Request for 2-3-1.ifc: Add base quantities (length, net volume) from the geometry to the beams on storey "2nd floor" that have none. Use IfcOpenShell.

First a look at what the model holds.

```python
import ifcopenshell
import ifcopenshell.util.element
import ifcopenshell.util.unit

model = ifcopenshell.open("2-3-1.ifc")
print(model.schema)
for unit_type in ("LENGTHUNIT", "AREAUNIT", "VOLUMEUNIT"):
    print(unit_type, ifcopenshell.util.unit.calculate_unit_scale(model, unit_type))
storey = next(s for s in model.by_type("IfcBuildingStorey") if s.Name == "2nd floor")
beams = [e for e in ifcopenshell.util.element.get_decomposition(storey) if e.is_a("IfcBeam")]
for e in sorted(beams, key=lambda e: e.id()):
    print(e.id(), e.is_a(), e.Name, list(ifcopenshell.util.element.get_psets(e, qtos_only=True)), sep=" | ")
```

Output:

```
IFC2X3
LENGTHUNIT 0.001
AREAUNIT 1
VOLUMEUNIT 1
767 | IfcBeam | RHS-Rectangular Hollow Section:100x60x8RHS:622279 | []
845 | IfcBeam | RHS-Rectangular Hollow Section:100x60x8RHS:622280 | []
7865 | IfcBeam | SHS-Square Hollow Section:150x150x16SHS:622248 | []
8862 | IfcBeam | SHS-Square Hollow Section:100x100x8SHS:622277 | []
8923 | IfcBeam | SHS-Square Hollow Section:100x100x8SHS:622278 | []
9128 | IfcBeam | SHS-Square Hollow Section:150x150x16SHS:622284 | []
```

```python
import ifcopenshell
import ifcopenshell.api.pset
import ifcopenshell.geom
import ifcopenshell.util.element
import ifcopenshell.util.shape
import ifcopenshell.util.unit

model = ifcopenshell.open("2-3-1.ifc")
unit_scale = ifcopenshell.util.unit.calculate_unit_scale(model)
volume_scale = ifcopenshell.util.unit.calculate_unit_scale(model, "VOLUMEUNIT")
settings = ifcopenshell.geom.settings()

storey = next(s for s in model.by_type("IfcBuildingStorey") if s.Name == "2nd floor")
beams = [e for e in ifcopenshell.util.element.get_decomposition(storey) if e.is_a("IfcBeam")]

for e in sorted(beams, key=lambda e: e.id()):
    if ifcopenshell.util.element.get_psets(e, qtos_only=True, should_inherit=False):
        continue
    # Geometry comes back in metres, in the element's own axes.
    shape = ifcopenshell.geom.create_shape(settings, e)
    values = {
        "Length": ifcopenshell.util.shape.get_max_xyz(shape.geometry) / unit_scale,
        "NetVolume": ifcopenshell.util.shape.get_volume(shape.geometry) / volume_scale,
    }
    qto = ifcopenshell.api.pset.add_qto(model, product=e, name="BaseQuantities")
    ifcopenshell.api.pset.edit_qto(model, qto=qto, properties=values)
    print(e.id(), {k: round(v, 3) for k, v in values.items()})

model.write("2-3-1_updated.ifc")
```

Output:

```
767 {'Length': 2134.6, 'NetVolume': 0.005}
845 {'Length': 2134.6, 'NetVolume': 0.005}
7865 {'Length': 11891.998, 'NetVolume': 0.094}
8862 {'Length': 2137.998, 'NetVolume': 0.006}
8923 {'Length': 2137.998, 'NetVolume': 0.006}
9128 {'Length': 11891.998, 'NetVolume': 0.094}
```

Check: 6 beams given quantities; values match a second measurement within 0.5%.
